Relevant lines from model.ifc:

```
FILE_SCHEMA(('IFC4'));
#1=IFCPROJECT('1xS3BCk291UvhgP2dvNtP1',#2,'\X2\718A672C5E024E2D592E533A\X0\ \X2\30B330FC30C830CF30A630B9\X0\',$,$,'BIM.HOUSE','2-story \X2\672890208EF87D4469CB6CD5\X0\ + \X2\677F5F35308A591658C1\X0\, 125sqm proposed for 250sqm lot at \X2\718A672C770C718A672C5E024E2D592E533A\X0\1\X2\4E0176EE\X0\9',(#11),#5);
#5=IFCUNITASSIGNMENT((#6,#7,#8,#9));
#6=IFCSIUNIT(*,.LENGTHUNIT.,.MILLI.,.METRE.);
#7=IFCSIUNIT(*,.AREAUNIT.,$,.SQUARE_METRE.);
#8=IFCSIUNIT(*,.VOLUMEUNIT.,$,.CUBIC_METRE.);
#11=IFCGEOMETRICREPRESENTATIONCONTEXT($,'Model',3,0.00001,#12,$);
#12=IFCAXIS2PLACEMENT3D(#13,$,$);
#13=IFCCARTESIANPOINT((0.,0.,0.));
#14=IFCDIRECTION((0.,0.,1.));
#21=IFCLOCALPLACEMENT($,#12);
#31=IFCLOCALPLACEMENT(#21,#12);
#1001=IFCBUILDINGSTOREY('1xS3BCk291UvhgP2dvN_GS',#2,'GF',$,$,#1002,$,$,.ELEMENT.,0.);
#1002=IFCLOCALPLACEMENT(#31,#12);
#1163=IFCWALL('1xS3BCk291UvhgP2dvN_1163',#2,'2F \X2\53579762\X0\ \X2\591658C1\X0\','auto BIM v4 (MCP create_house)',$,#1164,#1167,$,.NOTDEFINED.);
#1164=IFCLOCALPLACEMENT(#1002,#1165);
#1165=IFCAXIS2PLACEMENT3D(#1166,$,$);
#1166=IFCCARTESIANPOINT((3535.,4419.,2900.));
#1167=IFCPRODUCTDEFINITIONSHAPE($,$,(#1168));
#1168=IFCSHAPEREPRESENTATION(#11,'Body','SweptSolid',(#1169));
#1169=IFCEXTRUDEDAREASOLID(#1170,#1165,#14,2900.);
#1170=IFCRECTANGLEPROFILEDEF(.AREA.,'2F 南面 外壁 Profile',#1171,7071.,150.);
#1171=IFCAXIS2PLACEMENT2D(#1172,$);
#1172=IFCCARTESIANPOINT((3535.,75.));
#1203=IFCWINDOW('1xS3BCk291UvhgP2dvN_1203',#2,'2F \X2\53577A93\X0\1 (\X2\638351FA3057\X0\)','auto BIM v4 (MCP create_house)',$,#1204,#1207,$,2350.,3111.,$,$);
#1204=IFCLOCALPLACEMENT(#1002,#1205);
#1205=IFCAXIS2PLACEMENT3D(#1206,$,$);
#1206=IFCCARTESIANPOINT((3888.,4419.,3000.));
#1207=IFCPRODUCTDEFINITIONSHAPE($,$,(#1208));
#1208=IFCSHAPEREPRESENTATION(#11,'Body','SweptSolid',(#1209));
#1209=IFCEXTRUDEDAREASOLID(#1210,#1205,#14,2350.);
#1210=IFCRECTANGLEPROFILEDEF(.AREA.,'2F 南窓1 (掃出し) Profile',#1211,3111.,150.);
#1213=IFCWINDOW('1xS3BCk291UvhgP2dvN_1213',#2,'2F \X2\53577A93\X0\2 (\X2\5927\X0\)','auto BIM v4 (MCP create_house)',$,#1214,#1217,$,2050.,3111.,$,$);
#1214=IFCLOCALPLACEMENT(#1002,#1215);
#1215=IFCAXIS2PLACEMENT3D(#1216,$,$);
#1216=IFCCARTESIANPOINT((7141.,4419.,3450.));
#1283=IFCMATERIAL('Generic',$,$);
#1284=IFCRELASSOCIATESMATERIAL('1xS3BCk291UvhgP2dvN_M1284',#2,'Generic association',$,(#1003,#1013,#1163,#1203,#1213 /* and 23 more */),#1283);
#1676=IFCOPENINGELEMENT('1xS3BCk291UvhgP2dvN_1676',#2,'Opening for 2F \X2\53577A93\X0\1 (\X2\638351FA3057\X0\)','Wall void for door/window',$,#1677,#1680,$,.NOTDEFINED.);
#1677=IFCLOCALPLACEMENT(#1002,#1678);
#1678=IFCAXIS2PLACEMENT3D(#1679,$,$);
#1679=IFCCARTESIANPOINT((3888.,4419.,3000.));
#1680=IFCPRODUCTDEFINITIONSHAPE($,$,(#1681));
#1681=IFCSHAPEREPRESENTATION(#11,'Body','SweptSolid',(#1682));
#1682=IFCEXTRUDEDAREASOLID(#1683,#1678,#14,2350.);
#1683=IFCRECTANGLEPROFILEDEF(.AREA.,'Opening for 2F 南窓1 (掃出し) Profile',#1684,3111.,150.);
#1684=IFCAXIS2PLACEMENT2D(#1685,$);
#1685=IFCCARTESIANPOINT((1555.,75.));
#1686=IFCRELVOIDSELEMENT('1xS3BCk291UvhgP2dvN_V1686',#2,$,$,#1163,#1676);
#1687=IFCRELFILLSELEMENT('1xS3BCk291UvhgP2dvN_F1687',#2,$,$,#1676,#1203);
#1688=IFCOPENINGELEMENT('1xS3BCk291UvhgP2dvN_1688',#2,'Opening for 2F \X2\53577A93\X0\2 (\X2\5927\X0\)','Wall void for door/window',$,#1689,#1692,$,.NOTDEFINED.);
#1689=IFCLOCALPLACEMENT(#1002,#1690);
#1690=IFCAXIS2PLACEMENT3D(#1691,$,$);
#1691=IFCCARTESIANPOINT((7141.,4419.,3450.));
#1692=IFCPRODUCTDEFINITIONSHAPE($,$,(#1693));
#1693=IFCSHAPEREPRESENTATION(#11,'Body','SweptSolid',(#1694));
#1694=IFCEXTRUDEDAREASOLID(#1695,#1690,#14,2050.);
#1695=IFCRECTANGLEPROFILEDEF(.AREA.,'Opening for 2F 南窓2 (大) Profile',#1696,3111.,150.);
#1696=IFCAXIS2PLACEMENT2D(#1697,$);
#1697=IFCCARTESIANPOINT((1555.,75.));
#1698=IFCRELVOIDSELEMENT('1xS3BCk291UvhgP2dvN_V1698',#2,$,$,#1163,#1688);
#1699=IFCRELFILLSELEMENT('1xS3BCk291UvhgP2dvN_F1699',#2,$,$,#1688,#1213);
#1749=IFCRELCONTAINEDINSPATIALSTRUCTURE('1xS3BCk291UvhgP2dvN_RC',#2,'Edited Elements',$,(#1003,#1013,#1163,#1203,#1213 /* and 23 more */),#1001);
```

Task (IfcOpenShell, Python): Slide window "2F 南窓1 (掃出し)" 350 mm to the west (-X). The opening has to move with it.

```python
import ifcopenshell
import ifcopenshell.api.geometry
import ifcopenshell.util.placement
import ifcopenshell.util.unit

model = ifcopenshell.open("model.ifc")
unit_scale = ifcopenshell.util.unit.calculate_unit_scale(model)

window = model.by_guid("1xS3BCk291UvhgP2dvN_1203")
opening = window.FillsVoids[0].RelatingOpeningElement
wall = opening.VoidsElements[0].RelatingBuildingElement

wall_matrix = ifcopenshell.util.placement.get_local_placement(wall.ObjectPlacement)
shift = wall_matrix[:3, 0] * -0.35 / unit_scale
before = ifcopenshell.util.placement.get_local_placement(window.ObjectPlacement)[:3, 3].copy()

# The window is not placed relative to its opening, so move both.
for product in (opening, window):
    matrix = ifcopenshell.util.placement.get_local_placement(product.ObjectPlacement)
    matrix[:3, 3] += shift
    ifcopenshell.api.geometry.edit_object_placement(model, product=product, matrix=matrix, is_si=False)

after = ifcopenshell.util.placement.get_local_placement(window.ObjectPlacement)[:3, 3]
print("window moved by", (after - before).round(3) + 0.0)

model.write("model-out.ifc")
```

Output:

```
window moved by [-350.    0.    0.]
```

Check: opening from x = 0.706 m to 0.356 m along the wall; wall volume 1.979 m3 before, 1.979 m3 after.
